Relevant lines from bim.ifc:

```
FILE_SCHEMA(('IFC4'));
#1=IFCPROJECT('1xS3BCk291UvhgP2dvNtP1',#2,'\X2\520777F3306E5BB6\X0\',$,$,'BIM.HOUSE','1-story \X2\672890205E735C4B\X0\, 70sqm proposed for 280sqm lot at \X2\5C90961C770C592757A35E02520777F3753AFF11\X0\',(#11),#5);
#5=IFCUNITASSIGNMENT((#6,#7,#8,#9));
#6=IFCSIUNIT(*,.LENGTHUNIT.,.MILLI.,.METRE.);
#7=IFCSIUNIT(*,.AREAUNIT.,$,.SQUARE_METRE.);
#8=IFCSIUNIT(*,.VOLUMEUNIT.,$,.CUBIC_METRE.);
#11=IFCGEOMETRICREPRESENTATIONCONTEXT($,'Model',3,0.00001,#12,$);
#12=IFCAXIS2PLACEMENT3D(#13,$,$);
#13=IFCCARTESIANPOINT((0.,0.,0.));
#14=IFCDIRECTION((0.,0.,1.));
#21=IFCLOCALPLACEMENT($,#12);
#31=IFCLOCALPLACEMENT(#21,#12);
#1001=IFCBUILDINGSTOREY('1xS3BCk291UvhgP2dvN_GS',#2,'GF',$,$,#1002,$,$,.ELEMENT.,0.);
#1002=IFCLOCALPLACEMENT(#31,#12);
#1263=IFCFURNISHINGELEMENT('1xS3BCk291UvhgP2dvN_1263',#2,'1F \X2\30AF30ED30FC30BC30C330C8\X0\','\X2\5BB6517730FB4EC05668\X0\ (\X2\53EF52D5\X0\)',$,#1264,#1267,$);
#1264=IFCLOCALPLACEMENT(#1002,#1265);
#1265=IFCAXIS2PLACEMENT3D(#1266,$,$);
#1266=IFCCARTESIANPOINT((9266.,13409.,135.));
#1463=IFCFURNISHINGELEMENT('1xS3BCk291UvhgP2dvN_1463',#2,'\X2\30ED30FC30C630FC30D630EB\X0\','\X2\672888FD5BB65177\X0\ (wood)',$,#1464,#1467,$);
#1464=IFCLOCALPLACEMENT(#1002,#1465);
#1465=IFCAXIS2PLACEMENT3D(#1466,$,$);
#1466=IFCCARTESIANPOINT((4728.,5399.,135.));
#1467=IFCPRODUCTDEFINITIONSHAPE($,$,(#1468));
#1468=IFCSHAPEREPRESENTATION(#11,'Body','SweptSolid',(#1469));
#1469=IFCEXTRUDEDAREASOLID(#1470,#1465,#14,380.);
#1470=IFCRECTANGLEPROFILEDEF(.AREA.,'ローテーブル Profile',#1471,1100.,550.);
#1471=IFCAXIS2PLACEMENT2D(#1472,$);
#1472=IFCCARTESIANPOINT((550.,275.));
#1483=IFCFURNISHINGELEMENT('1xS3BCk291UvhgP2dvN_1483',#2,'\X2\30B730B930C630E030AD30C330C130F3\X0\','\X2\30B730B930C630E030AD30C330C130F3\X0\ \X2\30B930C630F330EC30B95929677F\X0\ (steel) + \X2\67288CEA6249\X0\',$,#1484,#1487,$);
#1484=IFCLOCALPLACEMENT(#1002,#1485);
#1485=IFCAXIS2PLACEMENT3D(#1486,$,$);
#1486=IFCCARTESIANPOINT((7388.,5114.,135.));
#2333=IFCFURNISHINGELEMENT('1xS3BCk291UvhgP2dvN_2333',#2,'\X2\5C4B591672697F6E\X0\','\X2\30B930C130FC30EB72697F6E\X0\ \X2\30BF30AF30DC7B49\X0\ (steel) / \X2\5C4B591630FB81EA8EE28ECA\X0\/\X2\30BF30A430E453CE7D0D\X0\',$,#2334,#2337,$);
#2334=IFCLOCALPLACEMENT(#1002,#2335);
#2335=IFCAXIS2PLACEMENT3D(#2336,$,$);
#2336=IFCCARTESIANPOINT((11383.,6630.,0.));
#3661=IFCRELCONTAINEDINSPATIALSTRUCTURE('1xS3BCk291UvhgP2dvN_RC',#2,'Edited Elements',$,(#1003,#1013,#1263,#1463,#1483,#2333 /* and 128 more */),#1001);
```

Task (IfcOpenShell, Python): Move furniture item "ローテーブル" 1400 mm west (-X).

```python
import ifcopenshell
import ifcopenshell.api.geometry
import ifcopenshell.util.placement

model = ifcopenshell.open("bim.ifc")

item = model.by_id(1463)
matrix = ifcopenshell.util.placement.get_local_placement(item.ObjectPlacement)
matrix[0, 3] -= 1400.0
ifcopenshell.api.geometry.edit_object_placement(model, product=item, matrix=matrix, is_si=False)

print(ifcopenshell.util.placement.get_local_placement(item.ObjectPlacement).round(3) + 0.0)

model.write("bim-out.ifc")
```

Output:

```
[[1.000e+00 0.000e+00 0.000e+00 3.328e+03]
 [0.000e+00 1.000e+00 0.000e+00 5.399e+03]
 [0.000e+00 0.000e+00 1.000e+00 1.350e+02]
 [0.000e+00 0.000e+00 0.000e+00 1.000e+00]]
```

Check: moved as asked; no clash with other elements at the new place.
